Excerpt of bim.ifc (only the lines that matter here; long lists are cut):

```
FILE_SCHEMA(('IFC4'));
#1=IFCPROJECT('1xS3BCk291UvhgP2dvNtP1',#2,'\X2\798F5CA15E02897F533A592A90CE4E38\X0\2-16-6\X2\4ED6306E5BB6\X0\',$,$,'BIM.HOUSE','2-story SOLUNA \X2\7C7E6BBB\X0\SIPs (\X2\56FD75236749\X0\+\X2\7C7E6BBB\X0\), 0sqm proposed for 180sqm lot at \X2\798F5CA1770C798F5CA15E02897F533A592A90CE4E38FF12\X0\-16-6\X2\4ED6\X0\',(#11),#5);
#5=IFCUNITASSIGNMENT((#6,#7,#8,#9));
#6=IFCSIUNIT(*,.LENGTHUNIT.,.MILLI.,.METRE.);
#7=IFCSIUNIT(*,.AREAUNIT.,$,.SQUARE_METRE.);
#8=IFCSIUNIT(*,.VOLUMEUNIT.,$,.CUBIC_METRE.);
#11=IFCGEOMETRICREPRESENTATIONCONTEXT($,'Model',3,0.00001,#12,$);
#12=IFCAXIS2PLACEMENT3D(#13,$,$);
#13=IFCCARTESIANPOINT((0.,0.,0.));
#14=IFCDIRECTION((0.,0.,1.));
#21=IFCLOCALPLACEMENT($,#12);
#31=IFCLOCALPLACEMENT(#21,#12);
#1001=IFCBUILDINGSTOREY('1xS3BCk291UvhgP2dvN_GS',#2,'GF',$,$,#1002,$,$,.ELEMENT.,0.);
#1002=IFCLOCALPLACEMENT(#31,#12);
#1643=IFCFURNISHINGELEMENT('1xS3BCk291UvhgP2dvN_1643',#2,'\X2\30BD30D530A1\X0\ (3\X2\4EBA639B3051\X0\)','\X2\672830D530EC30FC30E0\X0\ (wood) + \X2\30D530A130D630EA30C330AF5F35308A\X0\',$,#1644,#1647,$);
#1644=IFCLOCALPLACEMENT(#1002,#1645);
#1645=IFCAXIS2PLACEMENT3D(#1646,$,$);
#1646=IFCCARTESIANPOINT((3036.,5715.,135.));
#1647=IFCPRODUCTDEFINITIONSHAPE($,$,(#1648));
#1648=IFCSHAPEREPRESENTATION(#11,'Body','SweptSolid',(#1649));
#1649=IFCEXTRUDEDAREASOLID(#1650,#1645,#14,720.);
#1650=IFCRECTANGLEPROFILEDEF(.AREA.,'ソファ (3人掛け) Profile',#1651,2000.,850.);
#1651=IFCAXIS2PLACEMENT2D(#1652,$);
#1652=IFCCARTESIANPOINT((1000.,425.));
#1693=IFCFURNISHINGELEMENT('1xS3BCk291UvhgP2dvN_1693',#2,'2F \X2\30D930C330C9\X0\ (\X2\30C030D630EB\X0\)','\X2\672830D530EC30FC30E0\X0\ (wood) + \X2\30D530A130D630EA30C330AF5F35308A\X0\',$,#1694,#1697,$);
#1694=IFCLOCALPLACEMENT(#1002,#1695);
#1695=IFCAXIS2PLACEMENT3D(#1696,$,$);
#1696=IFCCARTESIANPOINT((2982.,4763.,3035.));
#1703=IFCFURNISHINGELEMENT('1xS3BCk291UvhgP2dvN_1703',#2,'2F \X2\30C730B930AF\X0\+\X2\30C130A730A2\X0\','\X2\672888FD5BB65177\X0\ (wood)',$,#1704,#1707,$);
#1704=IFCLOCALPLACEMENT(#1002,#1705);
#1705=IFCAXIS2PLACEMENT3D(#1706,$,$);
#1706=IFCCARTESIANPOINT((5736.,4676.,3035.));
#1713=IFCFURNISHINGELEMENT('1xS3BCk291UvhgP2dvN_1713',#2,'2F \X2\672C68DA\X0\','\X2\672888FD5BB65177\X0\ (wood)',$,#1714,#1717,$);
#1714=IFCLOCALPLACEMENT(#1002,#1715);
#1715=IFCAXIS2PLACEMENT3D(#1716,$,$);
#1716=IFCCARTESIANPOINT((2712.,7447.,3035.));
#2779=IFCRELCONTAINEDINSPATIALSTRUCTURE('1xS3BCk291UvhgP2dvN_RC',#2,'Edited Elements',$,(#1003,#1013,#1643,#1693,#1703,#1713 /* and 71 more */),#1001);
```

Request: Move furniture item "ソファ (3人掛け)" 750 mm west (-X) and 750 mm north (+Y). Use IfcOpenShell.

```python
import ifcopenshell
import ifcopenshell.api.geometry
import ifcopenshell.util.placement

model = ifcopenshell.open("bim.ifc")

item = model.by_guid("1xS3BCk291UvhgP2dvN_1643")
matrix = ifcopenshell.util.placement.get_local_placement(item.ObjectPlacement)
matrix[0, 3] -= 750.0
matrix[1, 3] += 750.0
ifcopenshell.api.geometry.edit_object_placement(model, product=item, matrix=matrix, is_si=False)

print(ifcopenshell.util.placement.get_local_placement(item.ObjectPlacement).round(3) + 0.0)

model.write("bim-out.ifc")
```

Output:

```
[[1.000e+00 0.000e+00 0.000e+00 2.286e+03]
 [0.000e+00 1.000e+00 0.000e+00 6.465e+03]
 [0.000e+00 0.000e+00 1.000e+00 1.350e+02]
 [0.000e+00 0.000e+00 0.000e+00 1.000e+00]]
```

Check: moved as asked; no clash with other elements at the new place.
